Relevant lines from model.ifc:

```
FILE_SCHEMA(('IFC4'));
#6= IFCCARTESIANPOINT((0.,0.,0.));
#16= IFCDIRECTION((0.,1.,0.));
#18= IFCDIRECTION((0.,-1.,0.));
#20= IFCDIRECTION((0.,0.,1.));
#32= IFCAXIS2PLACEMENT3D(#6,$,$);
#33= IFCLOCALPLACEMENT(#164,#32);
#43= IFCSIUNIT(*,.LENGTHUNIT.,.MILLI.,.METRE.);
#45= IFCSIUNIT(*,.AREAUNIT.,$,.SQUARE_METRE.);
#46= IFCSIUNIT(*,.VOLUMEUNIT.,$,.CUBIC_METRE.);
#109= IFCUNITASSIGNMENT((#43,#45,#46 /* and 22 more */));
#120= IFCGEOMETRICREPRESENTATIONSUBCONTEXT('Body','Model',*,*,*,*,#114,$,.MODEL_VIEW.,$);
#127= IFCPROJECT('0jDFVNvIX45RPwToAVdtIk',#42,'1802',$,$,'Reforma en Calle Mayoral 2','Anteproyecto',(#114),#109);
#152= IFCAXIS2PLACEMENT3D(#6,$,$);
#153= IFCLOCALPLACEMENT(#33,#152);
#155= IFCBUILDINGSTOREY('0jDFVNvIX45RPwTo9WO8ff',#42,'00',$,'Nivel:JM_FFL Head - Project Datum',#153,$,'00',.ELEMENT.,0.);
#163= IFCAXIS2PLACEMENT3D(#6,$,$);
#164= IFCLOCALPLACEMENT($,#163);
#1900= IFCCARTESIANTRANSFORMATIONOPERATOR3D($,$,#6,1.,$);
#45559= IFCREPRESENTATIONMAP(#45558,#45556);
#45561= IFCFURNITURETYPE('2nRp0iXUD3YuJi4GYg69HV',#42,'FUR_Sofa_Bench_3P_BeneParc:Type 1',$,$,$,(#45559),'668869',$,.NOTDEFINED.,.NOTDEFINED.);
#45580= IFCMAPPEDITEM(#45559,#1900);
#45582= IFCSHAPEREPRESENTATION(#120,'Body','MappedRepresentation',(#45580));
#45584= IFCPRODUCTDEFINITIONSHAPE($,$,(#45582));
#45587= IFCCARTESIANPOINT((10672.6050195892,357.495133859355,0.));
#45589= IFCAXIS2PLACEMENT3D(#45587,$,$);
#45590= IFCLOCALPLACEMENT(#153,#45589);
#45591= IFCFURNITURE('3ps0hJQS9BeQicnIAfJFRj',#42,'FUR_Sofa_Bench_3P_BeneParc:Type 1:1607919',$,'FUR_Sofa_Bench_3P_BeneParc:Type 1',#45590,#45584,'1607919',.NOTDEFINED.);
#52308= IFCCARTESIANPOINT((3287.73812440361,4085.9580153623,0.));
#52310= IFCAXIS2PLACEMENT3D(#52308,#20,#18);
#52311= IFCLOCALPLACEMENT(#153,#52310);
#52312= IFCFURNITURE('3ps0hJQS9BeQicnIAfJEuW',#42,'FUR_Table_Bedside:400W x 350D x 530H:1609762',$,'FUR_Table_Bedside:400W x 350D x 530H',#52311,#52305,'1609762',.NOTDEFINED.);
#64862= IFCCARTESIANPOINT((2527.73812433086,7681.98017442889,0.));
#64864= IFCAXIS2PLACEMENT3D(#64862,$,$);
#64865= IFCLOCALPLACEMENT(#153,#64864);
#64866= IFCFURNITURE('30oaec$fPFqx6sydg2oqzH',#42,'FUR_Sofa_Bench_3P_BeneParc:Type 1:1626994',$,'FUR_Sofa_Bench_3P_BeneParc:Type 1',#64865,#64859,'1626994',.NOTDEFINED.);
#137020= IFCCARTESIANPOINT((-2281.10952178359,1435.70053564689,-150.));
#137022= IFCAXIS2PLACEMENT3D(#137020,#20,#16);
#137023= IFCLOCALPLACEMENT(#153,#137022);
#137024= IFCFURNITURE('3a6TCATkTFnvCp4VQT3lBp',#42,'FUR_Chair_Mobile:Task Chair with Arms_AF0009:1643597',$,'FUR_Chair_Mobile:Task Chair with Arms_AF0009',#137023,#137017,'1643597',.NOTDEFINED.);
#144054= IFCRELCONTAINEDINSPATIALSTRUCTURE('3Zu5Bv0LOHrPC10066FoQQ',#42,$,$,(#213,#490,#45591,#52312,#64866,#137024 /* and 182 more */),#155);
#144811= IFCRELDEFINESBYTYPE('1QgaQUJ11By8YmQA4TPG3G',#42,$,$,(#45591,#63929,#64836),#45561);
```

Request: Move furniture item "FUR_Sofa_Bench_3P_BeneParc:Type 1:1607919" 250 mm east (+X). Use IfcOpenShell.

```python
import ifcopenshell
import ifcopenshell.api.geometry
import ifcopenshell.util.placement

model = ifcopenshell.open("model.ifc")

item = model.by_guid("3ps0hJQS9BeQicnIAfJFRj")
matrix = ifcopenshell.util.placement.get_local_placement(item.ObjectPlacement)
matrix[0, 3] += 250.0
ifcopenshell.api.geometry.edit_object_placement(model, product=item, matrix=matrix, is_si=False)

print(ifcopenshell.util.placement.get_local_placement(item.ObjectPlacement).round(3) + 0.0)

model.write("model_updated.ifc")
```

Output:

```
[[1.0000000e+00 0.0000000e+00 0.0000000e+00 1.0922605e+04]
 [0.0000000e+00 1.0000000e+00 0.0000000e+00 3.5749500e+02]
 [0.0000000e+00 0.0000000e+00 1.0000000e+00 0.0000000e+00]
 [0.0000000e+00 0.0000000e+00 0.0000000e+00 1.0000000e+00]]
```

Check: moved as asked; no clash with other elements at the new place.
